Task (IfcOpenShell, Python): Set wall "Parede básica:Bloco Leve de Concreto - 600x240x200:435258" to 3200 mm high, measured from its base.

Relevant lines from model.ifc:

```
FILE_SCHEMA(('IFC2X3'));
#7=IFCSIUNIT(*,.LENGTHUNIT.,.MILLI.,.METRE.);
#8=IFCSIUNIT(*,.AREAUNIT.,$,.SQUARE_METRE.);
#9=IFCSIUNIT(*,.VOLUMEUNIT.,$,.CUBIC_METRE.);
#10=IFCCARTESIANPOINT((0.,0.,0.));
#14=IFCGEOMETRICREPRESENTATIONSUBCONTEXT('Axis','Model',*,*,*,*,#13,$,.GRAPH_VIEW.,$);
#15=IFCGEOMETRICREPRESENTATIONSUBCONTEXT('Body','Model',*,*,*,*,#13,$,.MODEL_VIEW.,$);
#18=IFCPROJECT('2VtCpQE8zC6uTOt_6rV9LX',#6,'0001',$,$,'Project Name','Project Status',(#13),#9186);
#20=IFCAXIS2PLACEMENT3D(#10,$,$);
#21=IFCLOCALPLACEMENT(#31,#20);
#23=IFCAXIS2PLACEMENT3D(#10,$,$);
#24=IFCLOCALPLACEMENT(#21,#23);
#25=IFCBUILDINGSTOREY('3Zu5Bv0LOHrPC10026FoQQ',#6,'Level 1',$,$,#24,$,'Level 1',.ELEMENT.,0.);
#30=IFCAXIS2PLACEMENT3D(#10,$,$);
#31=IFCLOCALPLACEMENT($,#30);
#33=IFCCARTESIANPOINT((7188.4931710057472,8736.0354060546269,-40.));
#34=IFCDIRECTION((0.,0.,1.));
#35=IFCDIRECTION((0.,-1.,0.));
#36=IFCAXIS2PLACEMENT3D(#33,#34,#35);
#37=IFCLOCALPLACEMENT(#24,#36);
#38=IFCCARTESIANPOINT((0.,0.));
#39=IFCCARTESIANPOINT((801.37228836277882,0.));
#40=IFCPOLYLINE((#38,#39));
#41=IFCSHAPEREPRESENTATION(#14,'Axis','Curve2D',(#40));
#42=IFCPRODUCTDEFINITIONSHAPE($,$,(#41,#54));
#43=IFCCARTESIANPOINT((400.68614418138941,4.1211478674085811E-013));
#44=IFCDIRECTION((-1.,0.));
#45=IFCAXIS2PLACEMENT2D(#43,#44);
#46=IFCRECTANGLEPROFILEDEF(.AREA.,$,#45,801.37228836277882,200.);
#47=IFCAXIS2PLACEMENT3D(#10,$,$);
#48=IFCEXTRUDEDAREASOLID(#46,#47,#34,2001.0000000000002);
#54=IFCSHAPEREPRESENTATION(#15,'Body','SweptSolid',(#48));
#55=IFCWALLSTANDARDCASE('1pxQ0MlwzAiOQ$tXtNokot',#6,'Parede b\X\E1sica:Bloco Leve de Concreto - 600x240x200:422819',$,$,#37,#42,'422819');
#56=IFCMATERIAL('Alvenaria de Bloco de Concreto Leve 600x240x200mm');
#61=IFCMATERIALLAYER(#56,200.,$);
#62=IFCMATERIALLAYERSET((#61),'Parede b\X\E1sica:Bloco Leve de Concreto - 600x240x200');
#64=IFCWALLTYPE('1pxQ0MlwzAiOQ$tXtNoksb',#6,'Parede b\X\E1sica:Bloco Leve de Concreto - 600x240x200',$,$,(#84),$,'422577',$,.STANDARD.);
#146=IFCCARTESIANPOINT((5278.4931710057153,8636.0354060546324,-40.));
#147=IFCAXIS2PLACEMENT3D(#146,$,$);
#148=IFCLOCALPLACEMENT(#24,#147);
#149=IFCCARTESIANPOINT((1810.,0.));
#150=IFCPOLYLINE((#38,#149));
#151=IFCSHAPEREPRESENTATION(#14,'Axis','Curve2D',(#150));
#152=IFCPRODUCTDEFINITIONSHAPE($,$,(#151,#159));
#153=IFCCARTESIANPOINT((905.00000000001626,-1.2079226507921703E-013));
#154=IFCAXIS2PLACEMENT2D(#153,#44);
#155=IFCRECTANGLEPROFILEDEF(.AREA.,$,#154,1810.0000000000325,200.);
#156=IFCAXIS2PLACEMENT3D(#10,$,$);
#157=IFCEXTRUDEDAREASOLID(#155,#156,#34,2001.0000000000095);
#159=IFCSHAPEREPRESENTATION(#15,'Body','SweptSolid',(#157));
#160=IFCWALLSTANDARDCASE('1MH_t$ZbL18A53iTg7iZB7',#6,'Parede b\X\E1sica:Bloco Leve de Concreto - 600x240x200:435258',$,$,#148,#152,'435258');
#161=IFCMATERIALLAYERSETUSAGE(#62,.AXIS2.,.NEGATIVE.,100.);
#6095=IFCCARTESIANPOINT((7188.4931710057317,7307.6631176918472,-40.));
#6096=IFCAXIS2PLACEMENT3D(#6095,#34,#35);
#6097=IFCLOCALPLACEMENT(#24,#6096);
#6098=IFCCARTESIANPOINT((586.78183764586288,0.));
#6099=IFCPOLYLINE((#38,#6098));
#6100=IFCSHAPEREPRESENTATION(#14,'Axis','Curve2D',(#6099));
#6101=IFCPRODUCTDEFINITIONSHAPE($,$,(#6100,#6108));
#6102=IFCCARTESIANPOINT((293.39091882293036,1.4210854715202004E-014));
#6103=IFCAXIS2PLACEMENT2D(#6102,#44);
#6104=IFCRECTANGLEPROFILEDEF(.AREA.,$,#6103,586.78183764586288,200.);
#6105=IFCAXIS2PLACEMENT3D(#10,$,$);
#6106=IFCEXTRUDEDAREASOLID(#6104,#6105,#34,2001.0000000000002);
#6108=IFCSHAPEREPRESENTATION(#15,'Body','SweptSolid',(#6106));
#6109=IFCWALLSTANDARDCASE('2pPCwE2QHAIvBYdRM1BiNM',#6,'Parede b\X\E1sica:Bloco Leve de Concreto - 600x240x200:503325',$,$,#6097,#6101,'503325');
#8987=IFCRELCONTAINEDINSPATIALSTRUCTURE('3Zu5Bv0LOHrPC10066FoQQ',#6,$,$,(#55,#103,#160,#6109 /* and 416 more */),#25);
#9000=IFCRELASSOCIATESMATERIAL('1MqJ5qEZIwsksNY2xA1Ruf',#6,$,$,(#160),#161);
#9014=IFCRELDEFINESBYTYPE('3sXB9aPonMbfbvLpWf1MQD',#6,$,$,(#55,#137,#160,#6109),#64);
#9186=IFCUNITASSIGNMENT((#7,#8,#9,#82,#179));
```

```python
import ifcopenshell
import ifcopenshell.geom
import ifcopenshell.util.representation
import ifcopenshell.util.shape

model = ifcopenshell.open("model.ifc")
settings = ifcopenshell.geom.settings()


def volume(element):
    """Net volume in cubic metres, openings subtracted."""
    shape = ifcopenshell.geom.create_shape(settings, element)
    return ifcopenshell.util.shape.get_volume(shape.geometry)


wall = model.by_guid("1MH_t$ZbL18A53iTg7iZB7")
before = volume(wall)

body = ifcopenshell.util.representation.get_representation(wall, "Model", "Body")
solid = body.Items[0]
old_height = solid.Depth
solid.Depth = 3200.0
after = volume(wall)

print(f"height {old_height:g} -> {solid.Depth:g}, volume {before:.3f} -> {after:.3f} m3")

model.write("model_edited.ifc")
```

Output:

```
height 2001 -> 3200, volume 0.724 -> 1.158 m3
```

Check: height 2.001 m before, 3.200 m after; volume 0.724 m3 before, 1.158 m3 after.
